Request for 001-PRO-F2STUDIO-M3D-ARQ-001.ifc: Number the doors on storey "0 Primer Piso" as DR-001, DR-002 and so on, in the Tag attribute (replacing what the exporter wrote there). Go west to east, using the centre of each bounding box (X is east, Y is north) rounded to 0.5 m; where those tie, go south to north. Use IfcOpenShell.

First a look at what the model holds.

```python
import ifcopenshell
import ifcopenshell.util.element
import ifcopenshell.util.placement

model = ifcopenshell.open("001-PRO-F2STUDIO-M3D-ARQ-001.ifc")
print(model.schema)
storey = next(s for s in model.by_type("IfcBuildingStorey") if s.Name == "0 Primer Piso")
doors = [e for e in ifcopenshell.util.element.get_decomposition(storey) if e.is_a("IfcDoor")]
for e in sorted(doors, key=lambda e: e.id()):
    origin = ifcopenshell.util.placement.get_local_placement(e.ObjectPlacement)[:3, 3]
    print(e.id(), e.Tag, e.Name, origin.round(2) + 0.0, sep=" | ")
```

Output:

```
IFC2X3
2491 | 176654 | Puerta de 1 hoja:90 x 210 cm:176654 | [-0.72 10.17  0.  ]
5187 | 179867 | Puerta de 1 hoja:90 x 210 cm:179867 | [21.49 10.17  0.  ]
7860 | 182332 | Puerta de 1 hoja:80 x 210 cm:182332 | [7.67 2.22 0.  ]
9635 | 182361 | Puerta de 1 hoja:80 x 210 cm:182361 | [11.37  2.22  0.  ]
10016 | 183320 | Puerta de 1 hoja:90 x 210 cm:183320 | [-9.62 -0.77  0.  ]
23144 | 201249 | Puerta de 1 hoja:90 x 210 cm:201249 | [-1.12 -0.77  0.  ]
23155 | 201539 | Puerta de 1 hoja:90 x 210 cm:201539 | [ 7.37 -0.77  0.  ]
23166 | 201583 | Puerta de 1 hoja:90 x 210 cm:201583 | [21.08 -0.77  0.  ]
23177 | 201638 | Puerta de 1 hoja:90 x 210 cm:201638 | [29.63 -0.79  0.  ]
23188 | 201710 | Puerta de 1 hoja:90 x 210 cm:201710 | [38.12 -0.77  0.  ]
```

```python
import ifcopenshell
import ifcopenshell.geom
import ifcopenshell.util.element
import ifcopenshell.util.shape

model = ifcopenshell.open("001-PRO-F2STUDIO-M3D-ARQ-001.ifc")
settings = ifcopenshell.geom.settings()
settings.set("use-world-coords", True)


def centre(element):
    shape = ifcopenshell.geom.create_shape(settings, element)
    return ifcopenshell.util.shape.get_bbox_centroid(shape.geometry)


storey = next(s for s in model.by_type("IfcBuildingStorey") if s.Name == "0 Primer Piso")
doors = [e for e in ifcopenshell.util.element.get_decomposition(storey) if e.is_a("IfcDoor")]

# Insertion points can sit at a corner or the storey origin, so sort by the geometry (in metres).
centres = {e: centre(e) for e in doors}
doors.sort(key=lambda e: (round(centres[e][0] / 0.5), centres[e][1]))

for i, e in enumerate(doors, start=1):
    number = f"DR-0{i:02d}"
    e.Tag = number
    print(e.id(), number)

model.write("001-PRO-F2STUDIO-M3D-ARQ-001_v2.ifc")
```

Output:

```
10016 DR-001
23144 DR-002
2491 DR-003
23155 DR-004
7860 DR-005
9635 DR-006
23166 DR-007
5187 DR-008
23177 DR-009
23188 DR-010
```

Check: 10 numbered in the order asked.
